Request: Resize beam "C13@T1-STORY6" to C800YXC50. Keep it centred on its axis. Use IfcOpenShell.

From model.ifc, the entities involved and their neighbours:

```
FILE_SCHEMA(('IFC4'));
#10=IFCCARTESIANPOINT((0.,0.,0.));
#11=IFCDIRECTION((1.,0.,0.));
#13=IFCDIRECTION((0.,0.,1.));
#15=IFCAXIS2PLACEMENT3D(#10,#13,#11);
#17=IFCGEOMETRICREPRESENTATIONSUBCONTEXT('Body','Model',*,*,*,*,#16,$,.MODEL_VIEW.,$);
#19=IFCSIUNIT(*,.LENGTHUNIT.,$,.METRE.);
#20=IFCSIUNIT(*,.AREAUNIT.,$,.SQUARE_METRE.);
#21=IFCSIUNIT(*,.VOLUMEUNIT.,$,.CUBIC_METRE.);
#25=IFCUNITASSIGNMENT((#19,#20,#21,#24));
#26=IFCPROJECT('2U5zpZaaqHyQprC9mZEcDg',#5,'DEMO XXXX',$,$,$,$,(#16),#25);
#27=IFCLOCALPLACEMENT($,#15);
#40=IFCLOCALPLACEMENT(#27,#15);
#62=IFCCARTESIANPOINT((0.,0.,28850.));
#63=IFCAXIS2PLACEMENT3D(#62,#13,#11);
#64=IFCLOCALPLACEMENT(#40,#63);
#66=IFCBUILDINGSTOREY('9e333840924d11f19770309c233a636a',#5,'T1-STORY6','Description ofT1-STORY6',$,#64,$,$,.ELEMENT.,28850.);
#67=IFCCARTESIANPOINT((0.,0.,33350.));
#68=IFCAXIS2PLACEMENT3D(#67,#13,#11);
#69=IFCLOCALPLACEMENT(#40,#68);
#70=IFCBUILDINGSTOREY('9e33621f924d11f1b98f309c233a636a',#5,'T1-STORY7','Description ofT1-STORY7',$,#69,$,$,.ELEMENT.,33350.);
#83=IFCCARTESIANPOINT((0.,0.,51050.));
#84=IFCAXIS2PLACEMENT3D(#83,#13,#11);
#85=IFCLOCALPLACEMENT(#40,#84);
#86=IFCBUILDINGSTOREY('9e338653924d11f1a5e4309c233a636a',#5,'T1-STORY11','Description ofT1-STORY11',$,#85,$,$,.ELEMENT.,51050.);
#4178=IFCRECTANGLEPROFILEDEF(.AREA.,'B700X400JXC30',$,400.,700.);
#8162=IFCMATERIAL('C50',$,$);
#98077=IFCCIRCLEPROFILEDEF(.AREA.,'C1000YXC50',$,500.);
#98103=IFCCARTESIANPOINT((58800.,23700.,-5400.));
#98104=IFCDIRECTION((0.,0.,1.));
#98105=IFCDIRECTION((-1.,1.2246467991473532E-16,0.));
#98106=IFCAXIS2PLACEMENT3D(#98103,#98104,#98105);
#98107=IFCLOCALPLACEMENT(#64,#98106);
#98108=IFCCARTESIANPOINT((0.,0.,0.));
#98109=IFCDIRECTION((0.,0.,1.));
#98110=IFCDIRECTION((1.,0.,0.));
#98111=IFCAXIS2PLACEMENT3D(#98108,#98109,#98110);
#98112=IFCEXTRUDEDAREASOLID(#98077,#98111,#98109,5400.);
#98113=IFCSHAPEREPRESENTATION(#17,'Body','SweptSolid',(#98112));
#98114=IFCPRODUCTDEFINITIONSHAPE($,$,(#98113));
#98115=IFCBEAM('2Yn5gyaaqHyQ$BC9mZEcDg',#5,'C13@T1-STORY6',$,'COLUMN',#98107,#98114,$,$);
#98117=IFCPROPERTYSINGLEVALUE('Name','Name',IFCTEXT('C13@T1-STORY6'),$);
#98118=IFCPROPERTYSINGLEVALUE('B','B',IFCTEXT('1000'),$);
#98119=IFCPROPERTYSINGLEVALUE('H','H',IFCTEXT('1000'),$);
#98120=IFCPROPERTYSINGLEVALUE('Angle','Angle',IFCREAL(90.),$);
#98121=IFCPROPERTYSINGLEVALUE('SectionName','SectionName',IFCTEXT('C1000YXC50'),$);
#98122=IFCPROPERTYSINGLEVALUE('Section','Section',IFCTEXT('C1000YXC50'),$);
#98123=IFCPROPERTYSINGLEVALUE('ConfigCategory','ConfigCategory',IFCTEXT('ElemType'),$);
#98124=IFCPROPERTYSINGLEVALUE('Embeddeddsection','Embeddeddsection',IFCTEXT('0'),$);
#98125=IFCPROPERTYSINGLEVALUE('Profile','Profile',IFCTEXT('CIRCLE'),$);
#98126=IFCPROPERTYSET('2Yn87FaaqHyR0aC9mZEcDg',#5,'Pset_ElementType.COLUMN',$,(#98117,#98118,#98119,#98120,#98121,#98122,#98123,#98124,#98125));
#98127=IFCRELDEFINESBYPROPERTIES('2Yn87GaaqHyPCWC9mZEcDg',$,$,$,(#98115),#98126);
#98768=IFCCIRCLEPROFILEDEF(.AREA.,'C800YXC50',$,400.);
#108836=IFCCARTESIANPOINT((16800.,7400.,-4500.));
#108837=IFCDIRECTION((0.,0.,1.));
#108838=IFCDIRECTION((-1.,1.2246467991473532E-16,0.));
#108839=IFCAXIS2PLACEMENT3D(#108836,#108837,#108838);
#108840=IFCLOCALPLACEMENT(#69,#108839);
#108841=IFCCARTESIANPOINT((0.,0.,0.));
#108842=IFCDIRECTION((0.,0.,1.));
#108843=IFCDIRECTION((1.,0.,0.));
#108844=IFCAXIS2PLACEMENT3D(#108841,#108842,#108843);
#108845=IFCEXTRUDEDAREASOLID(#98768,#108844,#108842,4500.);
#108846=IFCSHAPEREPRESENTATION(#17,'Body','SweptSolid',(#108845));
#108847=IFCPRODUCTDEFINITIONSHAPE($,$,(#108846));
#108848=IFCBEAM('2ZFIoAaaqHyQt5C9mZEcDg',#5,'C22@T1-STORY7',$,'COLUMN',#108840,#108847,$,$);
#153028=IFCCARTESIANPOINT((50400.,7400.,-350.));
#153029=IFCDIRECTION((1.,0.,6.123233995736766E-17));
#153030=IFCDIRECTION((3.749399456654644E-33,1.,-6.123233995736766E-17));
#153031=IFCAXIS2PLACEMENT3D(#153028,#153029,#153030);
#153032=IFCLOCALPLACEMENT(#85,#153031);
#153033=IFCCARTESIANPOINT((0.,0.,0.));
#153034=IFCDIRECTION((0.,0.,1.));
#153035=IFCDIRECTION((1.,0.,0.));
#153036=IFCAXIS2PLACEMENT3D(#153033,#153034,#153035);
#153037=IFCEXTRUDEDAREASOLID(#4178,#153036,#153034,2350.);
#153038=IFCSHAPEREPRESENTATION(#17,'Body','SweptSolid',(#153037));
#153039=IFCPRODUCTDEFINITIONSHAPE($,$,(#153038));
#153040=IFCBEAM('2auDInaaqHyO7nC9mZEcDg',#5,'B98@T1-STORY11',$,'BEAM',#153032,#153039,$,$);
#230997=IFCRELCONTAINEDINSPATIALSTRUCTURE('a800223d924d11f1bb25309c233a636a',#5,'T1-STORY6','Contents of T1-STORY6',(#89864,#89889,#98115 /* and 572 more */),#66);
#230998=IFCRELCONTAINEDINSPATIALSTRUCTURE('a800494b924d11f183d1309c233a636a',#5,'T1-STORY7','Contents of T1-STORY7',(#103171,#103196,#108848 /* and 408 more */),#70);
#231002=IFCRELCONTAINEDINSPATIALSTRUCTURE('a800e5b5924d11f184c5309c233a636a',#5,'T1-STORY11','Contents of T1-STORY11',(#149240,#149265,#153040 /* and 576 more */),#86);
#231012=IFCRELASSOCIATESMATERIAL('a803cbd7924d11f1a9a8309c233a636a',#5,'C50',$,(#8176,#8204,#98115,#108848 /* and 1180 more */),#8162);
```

```python
import ifcopenshell
import ifcopenshell.api.pset
import ifcopenshell.util.element
import ifcopenshell.util.representation

model = ifcopenshell.open("model.ifc")

member = model.by_guid("2Yn5gyaaqHyQ$BC9mZEcDg")
source = next(p for p in model.by_type("IfcCircleProfileDef") if p.ProfileName == "C800YXC50")

body = ifcopenshell.util.representation.get_representation(member, "Model", "Body")
solid = body.Items[0]
old_profile = solid.SweptArea

# Copy the section's sizes but keep this member's own profile position.
profile = ifcopenshell.util.element.copy(model, source)
profile.Position = old_profile.Position
solid.SweptArea = profile
if not model.get_total_inverses(old_profile):
    ifcopenshell.util.element.remove_deep2(model, old_profile)
pset = model.by_id(ifcopenshell.util.element.get_pset(member, "Pset_ElementType.COLUMN", should_inherit=False)["id"])
ifcopenshell.api.pset.edit_pset(model, pset=pset, properties={"SectionName": "C800YXC50"})
pset = model.by_id(ifcopenshell.util.element.get_pset(member, "Pset_ElementType.COLUMN", should_inherit=False)["id"])
ifcopenshell.api.pset.edit_pset(model, pset=pset, properties={"Section": "C800YXC50"})

print(solid.SweptArea)

model.write("model_v2.ifc")
```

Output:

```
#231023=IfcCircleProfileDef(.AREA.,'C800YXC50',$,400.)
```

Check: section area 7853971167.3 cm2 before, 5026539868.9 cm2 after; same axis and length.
